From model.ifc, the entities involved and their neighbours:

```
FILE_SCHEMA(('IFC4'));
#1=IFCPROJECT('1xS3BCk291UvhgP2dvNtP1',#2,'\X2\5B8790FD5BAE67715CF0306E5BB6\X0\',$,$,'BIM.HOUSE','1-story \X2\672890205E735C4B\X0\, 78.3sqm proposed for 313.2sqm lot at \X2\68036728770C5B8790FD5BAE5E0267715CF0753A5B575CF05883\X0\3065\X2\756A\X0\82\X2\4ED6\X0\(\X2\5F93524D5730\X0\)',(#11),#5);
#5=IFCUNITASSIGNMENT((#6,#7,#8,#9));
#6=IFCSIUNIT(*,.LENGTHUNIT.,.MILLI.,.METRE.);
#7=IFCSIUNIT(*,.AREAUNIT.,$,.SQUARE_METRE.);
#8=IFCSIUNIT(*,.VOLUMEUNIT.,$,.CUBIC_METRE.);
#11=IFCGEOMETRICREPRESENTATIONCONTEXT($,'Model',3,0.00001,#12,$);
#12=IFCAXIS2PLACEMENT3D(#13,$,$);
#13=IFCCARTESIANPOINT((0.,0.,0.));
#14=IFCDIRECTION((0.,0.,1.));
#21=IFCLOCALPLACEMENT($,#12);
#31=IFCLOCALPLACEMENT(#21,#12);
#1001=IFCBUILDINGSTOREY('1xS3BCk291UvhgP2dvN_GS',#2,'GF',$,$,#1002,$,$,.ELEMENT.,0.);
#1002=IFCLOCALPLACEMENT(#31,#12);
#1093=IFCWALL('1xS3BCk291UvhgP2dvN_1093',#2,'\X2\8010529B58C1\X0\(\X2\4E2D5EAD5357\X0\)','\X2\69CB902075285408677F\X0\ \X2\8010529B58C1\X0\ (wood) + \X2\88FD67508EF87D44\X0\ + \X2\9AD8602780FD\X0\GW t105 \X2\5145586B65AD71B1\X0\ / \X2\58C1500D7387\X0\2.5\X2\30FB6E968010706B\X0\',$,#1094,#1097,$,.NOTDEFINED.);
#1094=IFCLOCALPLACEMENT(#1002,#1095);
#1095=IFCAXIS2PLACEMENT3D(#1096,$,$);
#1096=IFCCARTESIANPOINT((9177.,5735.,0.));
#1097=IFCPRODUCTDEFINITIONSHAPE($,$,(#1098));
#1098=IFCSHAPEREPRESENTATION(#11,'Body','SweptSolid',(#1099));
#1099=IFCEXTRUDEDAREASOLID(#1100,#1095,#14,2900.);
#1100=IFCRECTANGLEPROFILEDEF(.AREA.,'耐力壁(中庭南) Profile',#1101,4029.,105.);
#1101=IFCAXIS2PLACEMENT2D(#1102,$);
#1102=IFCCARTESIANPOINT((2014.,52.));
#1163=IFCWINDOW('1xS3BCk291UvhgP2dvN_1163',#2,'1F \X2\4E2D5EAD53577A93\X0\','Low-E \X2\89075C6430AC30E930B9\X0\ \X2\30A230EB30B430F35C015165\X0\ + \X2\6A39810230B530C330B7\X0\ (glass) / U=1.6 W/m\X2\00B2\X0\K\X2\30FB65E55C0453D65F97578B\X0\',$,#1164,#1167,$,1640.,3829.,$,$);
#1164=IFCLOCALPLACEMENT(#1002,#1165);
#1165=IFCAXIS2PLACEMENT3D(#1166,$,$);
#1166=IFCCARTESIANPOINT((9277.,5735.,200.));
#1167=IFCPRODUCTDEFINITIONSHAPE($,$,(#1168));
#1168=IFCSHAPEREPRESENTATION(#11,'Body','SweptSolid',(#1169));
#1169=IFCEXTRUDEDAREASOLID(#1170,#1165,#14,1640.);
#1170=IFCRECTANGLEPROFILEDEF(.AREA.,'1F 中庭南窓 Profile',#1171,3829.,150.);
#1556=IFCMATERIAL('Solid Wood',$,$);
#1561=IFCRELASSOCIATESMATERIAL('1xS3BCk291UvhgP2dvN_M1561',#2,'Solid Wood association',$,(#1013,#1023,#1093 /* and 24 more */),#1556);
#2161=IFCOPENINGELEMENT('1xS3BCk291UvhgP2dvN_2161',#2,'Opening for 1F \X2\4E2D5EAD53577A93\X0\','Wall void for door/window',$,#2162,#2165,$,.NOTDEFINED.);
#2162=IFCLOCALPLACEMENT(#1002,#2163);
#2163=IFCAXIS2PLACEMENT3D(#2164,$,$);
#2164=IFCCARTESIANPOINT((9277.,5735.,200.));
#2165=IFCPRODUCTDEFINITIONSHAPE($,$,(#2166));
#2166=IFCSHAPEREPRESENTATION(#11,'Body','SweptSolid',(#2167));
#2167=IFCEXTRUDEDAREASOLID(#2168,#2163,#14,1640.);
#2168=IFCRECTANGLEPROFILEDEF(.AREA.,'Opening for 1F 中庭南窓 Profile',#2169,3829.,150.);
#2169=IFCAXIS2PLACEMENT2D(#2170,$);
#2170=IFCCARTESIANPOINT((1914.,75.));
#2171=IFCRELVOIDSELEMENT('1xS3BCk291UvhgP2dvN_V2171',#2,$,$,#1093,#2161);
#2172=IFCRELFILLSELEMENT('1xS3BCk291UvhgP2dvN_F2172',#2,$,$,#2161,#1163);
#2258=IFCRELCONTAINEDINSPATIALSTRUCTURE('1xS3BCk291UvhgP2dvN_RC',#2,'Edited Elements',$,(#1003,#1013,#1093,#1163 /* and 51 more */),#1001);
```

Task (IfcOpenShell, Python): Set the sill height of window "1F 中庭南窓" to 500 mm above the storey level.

```python
import numpy as np
import ifcopenshell
import ifcopenshell.api.geometry
import ifcopenshell.geom
import ifcopenshell.util.element
import ifcopenshell.util.placement
import ifcopenshell.util.shape
import ifcopenshell.util.unit

model = ifcopenshell.open("model.ifc")
unit_scale = ifcopenshell.util.unit.calculate_unit_scale(model)

window = model.by_guid("1xS3BCk291UvhgP2dvN_1163")
opening = window.FillsVoids[0].RelatingOpeningElement
storey = ifcopenshell.util.element.get_container(window, ifc_class="IfcBuildingStorey")
level = ifcopenshell.util.placement.get_local_placement(storey.ObjectPlacement)[2, 3]

# The opening's origin need not be at the sill, so measure its lowest point.
shape = ifcopenshell.geom.create_shape(ifcopenshell.geom.settings(), opening)
bottom = ifcopenshell.util.shape.get_shape_bottom_elevation(shape, shape.geometry) / unit_scale
dz = level + 500.0 - bottom

shift = np.array([0.0, 0.0, dz])
# The window is not placed relative to its opening, so move both.
for product in (opening, window):
    matrix = ifcopenshell.util.placement.get_local_placement(product.ObjectPlacement)
    matrix[:3, 3] += shift
    ifcopenshell.api.geometry.edit_object_placement(model, product=product, matrix=matrix, is_si=False)

print(f"moved by {dz * unit_scale:+.3f} m")

model.write("model_rev.ifc")
```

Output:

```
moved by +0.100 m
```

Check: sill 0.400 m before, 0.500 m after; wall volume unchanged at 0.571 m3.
